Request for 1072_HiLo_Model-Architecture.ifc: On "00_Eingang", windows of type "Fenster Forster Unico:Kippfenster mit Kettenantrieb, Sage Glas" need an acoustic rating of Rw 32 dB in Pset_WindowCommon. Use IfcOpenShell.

First a look at what the model holds.

```python
import ifcopenshell
import ifcopenshell.util.element

model = ifcopenshell.open("1072_HiLo_Model-Architecture.ifc")
print(model.schema)
storey = next(s for s in model.by_type("IfcBuildingStorey") if s.Name == "00_Eingang")
windows = [e for e in ifcopenshell.util.element.get_decomposition(storey) if e.is_a("IfcWindow")]
seen = {}
for e in windows:
    element_type = ifcopenshell.util.element.get_type(e)
    key = (element_type.Name if element_type != e and element_type else None, ifcopenshell.util.element.get_pset(e, "Pset_WindowCommon", "AcousticRating"))
    seen[key] = seen.get(key, 0) + 1
for (name, value), count in sorted(seen.items(), key=str):
    print(count, "x", name, "|", value)
```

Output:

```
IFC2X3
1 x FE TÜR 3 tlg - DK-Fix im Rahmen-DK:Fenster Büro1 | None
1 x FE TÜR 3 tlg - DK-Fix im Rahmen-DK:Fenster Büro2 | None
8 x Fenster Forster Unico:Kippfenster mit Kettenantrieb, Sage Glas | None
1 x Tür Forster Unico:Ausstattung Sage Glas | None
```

```python
import ifcopenshell
import ifcopenshell.api.pset
import ifcopenshell.util.element

model = ifcopenshell.open("1072_HiLo_Model-Architecture.ifc")

storey = next(s for s in model.by_type("IfcBuildingStorey") if s.Name == "00_Eingang")
windows = [e for e in ifcopenshell.util.element.get_decomposition(storey) if e.is_a("IfcWindow")]

count = 0
for e in windows:
    element_type = ifcopenshell.util.element.get_type(e)
    if element_type in (None, e) or element_type.Name != "Fenster Forster Unico:Kippfenster mit Kettenantrieb, Sage Glas":
        continue
    # add_pset returns the element's existing set when there is one.
    pset = ifcopenshell.api.pset.add_pset(model, product=e, name="Pset_WindowCommon")
    ifcopenshell.api.pset.edit_pset(model, pset=pset, properties={"AcousticRating": "Rw 32 dB"})
    count += 1

print(count, "windows updated")

model.write("1072_HiLo_Model-Architecture-out.ifc")
```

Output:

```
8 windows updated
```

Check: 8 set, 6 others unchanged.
